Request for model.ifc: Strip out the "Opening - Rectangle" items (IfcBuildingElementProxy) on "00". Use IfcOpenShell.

First a look at what the model holds.

```python
import ifcopenshell
import ifcopenshell.util.element

model = ifcopenshell.open("model.ifc")
print(model.schema)
storey = next(s for s in model.by_type("IfcBuildingStorey") if s.Name == "00")
proxies = [e for e in ifcopenshell.util.element.get_decomposition(storey) if e.is_a("IfcBuildingElementProxy")]
seen = {}
for e in proxies:
    element_type = ifcopenshell.util.element.get_type(e)
    name = element_type.Name if element_type not in (None, e) else None
    seen[name] = seen.get(name, 0) + 1
for name, count in sorted(seen.items(), key=str):
    print(count, "x", name)
```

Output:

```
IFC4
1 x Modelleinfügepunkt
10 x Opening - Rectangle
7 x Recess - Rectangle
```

```python
import ifcopenshell
import ifcopenshell.api.root
import ifcopenshell.util.element

model = ifcopenshell.open("model.ifc")

storey = next(s for s in model.by_type("IfcBuildingStorey") if s.Name == "00")
proxies = [e for e in ifcopenshell.util.element.get_decomposition(storey) if e.is_a("IfcBuildingElementProxy")]
targets = [e for e in proxies if (t := ifcopenshell.util.element.get_type(e)) not in (None, e) and t.Name == "Opening - Rectangle"]

for e in targets:
    ifcopenshell.api.root.remove_product(model, product=e)
print(len(targets), "removed")

model.write("model_edited.ifc")
```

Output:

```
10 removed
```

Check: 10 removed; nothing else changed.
